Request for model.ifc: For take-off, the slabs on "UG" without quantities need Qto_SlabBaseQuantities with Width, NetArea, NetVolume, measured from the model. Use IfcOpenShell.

First a look at what the model holds.

```python
import ifcopenshell
import ifcopenshell.util.element
import ifcopenshell.util.unit

model = ifcopenshell.open("model.ifc")
print(model.schema)
for unit_type in ("LENGTHUNIT", "AREAUNIT", "VOLUMEUNIT"):
    print(unit_type, ifcopenshell.util.unit.calculate_unit_scale(model, unit_type))
storey = next(s for s in model.by_type("IfcBuildingStorey") if s.Name == "UG")
slabs = [e for e in ifcopenshell.util.element.get_decomposition(storey) if e.is_a("IfcSlab")]
for e in sorted(slabs, key=lambda e: e.id()):
    print(e.id(), e.is_a(), e.Name, list(ifcopenshell.util.element.get_psets(e, qtos_only=True)), sep=" | ")
```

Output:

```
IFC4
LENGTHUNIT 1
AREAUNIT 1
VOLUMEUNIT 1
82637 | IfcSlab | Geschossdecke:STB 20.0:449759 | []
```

```python
import ifcopenshell
import ifcopenshell.api.pset
import ifcopenshell.geom
import ifcopenshell.util.element
import ifcopenshell.util.shape
import ifcopenshell.util.unit

model = ifcopenshell.open("model.ifc")
unit_scale = ifcopenshell.util.unit.calculate_unit_scale(model)
area_scale = ifcopenshell.util.unit.calculate_unit_scale(model, "AREAUNIT")
volume_scale = ifcopenshell.util.unit.calculate_unit_scale(model, "VOLUMEUNIT")
settings = ifcopenshell.geom.settings()

storey = next(s for s in model.by_type("IfcBuildingStorey") if s.Name == "UG")
slabs = [e for e in ifcopenshell.util.element.get_decomposition(storey) if e.is_a("IfcSlab")]

for e in sorted(slabs, key=lambda e: e.id()):
    if ifcopenshell.util.element.get_psets(e, qtos_only=True, should_inherit=False):
        continue
    # Geometry comes back in metres, in the element's own axes.
    shape = ifcopenshell.geom.create_shape(settings, e)
    values = {
        "Width": ifcopenshell.util.shape.get_z(shape.geometry) / unit_scale,
        "NetArea": ifcopenshell.util.shape.get_footprint_area(shape.geometry) / area_scale,
        "NetVolume": ifcopenshell.util.shape.get_volume(shape.geometry) / volume_scale,
    }
    qto = ifcopenshell.api.pset.add_qto(model, product=e, name="Qto_SlabBaseQuantities")
    ifcopenshell.api.pset.edit_qto(model, qto=qto, properties=values)
    print(e.id(), {k: round(v, 3) for k, v in values.items()})

model.write("model_rev.ifc")
```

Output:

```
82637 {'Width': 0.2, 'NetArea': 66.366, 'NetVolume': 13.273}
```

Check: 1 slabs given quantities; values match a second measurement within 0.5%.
